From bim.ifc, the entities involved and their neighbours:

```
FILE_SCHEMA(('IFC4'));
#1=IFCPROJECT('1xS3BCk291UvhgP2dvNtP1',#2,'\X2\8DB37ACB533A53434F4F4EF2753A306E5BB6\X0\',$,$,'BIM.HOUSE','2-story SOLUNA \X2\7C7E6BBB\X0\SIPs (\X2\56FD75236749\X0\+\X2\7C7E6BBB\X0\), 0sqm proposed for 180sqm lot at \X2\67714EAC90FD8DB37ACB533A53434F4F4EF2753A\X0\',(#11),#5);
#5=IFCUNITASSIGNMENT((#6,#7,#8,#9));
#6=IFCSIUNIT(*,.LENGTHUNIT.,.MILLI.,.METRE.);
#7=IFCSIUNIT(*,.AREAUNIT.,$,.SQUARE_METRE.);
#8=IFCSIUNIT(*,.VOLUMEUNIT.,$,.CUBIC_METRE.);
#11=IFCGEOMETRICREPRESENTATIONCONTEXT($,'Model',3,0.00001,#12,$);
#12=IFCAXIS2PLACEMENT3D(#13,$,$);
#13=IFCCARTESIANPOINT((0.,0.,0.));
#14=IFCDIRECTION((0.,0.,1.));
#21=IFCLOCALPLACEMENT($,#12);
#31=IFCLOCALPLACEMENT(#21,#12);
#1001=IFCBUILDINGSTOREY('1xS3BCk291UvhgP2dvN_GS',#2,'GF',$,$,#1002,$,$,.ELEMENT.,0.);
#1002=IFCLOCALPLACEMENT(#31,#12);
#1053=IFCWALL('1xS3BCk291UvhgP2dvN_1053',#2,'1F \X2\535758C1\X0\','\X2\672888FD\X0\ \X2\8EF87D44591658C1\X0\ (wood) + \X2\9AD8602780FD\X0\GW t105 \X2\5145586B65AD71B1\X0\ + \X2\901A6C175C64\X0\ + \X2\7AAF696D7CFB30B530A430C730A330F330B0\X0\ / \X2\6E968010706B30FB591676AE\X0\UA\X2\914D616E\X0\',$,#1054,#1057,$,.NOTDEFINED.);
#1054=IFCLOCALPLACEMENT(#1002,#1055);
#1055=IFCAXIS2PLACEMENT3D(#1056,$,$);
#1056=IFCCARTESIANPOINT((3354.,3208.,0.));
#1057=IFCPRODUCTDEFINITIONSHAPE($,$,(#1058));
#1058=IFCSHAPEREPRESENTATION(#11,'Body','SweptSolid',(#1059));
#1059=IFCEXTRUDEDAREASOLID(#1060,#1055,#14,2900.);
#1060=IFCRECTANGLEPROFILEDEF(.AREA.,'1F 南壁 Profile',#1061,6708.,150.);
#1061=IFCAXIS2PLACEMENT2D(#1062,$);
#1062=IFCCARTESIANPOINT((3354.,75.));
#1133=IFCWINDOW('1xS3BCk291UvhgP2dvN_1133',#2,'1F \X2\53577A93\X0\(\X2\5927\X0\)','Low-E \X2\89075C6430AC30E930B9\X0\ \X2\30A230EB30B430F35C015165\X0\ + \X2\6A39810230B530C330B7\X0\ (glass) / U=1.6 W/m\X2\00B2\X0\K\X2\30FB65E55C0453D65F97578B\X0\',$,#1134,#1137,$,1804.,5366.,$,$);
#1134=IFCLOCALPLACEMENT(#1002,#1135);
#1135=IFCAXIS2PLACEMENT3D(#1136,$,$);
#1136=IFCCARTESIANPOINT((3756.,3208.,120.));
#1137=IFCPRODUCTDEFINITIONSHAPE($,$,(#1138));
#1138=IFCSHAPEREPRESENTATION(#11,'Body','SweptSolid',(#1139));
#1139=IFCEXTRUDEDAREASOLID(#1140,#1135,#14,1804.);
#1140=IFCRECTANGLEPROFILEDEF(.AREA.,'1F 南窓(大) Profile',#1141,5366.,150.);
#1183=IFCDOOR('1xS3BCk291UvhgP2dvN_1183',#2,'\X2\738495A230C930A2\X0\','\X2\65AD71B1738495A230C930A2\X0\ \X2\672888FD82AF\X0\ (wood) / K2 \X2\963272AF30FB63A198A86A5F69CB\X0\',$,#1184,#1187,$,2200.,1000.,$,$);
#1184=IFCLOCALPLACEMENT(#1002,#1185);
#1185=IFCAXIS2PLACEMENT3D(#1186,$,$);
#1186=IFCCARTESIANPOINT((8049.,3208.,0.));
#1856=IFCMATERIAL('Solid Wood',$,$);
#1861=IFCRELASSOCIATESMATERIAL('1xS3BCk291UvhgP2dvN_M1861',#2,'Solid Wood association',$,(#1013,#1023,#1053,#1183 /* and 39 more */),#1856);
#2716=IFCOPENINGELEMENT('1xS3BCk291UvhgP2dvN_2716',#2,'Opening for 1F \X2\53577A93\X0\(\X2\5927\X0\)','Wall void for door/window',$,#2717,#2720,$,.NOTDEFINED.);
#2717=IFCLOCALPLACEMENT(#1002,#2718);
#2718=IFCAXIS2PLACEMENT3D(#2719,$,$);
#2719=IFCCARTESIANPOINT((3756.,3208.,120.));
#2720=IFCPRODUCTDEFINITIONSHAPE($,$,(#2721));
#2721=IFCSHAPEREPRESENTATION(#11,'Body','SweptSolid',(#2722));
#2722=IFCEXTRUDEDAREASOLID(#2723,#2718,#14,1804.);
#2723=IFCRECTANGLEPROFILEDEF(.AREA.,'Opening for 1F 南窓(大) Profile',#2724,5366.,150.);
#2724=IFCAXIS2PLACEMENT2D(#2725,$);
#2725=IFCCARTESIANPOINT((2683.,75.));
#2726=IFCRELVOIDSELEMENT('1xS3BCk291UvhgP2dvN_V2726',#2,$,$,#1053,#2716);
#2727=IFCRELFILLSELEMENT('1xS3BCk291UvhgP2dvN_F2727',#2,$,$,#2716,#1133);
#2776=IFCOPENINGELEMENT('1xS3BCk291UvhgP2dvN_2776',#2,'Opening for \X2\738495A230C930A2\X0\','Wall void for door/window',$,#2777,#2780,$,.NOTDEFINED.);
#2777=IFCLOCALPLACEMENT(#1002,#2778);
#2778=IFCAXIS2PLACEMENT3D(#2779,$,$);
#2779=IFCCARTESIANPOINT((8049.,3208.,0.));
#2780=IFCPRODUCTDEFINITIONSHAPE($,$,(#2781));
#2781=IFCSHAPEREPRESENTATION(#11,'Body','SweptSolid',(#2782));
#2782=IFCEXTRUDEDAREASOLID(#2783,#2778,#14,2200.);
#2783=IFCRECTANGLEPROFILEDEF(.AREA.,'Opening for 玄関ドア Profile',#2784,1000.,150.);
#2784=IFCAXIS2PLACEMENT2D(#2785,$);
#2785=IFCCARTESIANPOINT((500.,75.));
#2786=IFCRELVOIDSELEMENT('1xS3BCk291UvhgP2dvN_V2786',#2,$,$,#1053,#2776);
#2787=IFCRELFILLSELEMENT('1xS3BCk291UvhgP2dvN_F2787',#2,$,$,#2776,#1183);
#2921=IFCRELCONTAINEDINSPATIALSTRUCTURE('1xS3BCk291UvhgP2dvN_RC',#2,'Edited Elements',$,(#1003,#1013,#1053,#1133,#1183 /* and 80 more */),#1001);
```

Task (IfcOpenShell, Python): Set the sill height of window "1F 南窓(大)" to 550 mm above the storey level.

```python
import numpy as np
import ifcopenshell
import ifcopenshell.api.geometry
import ifcopenshell.geom
import ifcopenshell.util.element
import ifcopenshell.util.placement
import ifcopenshell.util.shape
import ifcopenshell.util.unit

model = ifcopenshell.open("bim.ifc")
unit_scale = ifcopenshell.util.unit.calculate_unit_scale(model)

window = model.by_guid("1xS3BCk291UvhgP2dvN_1133")
opening = window.FillsVoids[0].RelatingOpeningElement
storey = ifcopenshell.util.element.get_container(window, ifc_class="IfcBuildingStorey")
level = ifcopenshell.util.placement.get_local_placement(storey.ObjectPlacement)[2, 3]

# The opening's origin need not be at the sill, so measure its lowest point.
shape = ifcopenshell.geom.create_shape(ifcopenshell.geom.settings(), opening)
bottom = ifcopenshell.util.shape.get_shape_bottom_elevation(shape, shape.geometry) / unit_scale
dz = level + 0.55 / unit_scale - bottom

shift = np.array([0.0, 0.0, dz])
# The window is not placed relative to its opening, so move both.
for product in (opening, window):
    matrix = ifcopenshell.util.placement.get_local_placement(product.ObjectPlacement)
    matrix[:3, 3] += shift
    ifcopenshell.api.geometry.edit_object_placement(model, product=product, matrix=matrix, is_si=False)

print(f"moved by {dz * unit_scale:+.3f} m")

model.write("bim_v2.ifc")
```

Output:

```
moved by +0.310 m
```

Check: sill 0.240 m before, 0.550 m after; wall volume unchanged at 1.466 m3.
